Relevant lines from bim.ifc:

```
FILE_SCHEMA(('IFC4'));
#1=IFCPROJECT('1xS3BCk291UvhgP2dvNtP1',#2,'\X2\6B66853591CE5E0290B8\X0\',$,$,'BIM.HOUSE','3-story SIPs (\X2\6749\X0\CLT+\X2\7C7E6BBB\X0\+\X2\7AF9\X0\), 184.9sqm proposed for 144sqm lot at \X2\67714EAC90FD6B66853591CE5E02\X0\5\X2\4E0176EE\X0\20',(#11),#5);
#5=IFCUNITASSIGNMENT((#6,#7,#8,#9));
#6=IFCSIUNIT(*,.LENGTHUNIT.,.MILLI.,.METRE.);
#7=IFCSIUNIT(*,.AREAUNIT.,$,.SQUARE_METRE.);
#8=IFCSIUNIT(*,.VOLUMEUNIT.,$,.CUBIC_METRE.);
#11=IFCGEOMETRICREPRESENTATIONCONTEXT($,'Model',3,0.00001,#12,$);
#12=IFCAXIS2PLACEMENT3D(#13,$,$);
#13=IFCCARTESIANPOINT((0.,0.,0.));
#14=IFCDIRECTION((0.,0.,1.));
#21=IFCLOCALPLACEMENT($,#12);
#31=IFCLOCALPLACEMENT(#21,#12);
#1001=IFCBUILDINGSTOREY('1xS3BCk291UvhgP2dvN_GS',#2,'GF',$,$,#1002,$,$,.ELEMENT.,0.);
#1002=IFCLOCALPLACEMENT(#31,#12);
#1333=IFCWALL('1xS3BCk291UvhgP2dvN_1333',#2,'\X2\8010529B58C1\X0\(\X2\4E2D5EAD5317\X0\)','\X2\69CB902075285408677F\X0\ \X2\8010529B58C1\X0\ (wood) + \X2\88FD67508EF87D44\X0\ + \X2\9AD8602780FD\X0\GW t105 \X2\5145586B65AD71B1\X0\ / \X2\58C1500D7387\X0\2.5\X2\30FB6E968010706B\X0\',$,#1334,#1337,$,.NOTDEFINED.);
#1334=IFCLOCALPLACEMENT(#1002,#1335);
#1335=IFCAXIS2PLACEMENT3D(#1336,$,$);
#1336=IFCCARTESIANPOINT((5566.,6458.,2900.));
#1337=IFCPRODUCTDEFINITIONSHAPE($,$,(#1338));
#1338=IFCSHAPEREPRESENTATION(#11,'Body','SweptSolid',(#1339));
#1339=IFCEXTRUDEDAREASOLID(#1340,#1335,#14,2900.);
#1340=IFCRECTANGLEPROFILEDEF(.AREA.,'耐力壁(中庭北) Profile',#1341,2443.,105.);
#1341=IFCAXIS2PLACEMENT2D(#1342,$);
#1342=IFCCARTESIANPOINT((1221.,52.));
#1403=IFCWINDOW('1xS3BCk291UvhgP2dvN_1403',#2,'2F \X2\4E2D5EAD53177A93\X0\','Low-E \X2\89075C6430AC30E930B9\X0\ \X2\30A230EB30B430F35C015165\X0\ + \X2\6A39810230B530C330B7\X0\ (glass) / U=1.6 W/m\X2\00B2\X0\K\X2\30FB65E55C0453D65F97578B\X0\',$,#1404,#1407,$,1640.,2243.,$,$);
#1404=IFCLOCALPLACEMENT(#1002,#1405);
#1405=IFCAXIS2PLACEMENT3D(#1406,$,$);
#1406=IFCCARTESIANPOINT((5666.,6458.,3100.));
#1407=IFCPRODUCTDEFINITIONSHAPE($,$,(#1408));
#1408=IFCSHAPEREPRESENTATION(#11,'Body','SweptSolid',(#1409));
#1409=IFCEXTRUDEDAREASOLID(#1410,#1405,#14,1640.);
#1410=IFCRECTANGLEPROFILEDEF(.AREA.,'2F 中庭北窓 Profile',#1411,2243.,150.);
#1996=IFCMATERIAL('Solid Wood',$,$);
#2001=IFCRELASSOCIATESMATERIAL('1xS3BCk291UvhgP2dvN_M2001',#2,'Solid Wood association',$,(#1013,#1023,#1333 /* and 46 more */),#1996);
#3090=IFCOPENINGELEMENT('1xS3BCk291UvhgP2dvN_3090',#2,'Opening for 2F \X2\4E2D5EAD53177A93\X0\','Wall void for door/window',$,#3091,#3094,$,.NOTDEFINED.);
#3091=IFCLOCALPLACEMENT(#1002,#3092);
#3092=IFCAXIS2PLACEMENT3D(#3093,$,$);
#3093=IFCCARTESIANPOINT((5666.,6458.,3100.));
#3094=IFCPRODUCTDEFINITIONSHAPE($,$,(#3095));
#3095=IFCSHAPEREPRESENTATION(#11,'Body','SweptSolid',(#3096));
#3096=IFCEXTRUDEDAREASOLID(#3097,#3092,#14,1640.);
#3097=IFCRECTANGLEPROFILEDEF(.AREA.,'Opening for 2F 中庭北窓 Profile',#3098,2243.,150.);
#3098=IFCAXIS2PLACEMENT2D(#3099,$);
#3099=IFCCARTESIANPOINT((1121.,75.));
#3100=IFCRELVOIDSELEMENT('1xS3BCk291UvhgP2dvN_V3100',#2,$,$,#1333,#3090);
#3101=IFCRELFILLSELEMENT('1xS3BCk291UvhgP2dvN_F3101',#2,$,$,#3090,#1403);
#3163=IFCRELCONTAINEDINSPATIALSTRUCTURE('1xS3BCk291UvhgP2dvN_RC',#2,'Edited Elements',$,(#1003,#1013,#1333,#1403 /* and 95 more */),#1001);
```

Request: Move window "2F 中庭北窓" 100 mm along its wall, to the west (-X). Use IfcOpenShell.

```python
import ifcopenshell
import ifcopenshell.api.geometry
import ifcopenshell.util.placement
import ifcopenshell.util.unit

model = ifcopenshell.open("bim.ifc")
unit_scale = ifcopenshell.util.unit.calculate_unit_scale(model)

window = model.by_guid("1xS3BCk291UvhgP2dvN_1403")
opening = window.FillsVoids[0].RelatingOpeningElement
wall = opening.VoidsElements[0].RelatingBuildingElement

wall_matrix = ifcopenshell.util.placement.get_local_placement(wall.ObjectPlacement)
shift = wall_matrix[:3, 0] * -0.1 / unit_scale
before = ifcopenshell.util.placement.get_local_placement(window.ObjectPlacement)[:3, 3].copy()

# The window is not placed relative to its opening, so move both.
for product in (opening, window):
    matrix = ifcopenshell.util.placement.get_local_placement(product.ObjectPlacement)
    matrix[:3, 3] += shift
    ifcopenshell.api.geometry.edit_object_placement(model, product=product, matrix=matrix, is_si=False)

after = ifcopenshell.util.placement.get_local_placement(window.ObjectPlacement)[:3, 3]
print("window moved by", (after - before).round(3) + 0.0)

model.write("bim_updated.ifc")
```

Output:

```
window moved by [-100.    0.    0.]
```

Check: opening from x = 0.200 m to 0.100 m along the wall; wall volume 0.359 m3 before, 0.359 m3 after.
